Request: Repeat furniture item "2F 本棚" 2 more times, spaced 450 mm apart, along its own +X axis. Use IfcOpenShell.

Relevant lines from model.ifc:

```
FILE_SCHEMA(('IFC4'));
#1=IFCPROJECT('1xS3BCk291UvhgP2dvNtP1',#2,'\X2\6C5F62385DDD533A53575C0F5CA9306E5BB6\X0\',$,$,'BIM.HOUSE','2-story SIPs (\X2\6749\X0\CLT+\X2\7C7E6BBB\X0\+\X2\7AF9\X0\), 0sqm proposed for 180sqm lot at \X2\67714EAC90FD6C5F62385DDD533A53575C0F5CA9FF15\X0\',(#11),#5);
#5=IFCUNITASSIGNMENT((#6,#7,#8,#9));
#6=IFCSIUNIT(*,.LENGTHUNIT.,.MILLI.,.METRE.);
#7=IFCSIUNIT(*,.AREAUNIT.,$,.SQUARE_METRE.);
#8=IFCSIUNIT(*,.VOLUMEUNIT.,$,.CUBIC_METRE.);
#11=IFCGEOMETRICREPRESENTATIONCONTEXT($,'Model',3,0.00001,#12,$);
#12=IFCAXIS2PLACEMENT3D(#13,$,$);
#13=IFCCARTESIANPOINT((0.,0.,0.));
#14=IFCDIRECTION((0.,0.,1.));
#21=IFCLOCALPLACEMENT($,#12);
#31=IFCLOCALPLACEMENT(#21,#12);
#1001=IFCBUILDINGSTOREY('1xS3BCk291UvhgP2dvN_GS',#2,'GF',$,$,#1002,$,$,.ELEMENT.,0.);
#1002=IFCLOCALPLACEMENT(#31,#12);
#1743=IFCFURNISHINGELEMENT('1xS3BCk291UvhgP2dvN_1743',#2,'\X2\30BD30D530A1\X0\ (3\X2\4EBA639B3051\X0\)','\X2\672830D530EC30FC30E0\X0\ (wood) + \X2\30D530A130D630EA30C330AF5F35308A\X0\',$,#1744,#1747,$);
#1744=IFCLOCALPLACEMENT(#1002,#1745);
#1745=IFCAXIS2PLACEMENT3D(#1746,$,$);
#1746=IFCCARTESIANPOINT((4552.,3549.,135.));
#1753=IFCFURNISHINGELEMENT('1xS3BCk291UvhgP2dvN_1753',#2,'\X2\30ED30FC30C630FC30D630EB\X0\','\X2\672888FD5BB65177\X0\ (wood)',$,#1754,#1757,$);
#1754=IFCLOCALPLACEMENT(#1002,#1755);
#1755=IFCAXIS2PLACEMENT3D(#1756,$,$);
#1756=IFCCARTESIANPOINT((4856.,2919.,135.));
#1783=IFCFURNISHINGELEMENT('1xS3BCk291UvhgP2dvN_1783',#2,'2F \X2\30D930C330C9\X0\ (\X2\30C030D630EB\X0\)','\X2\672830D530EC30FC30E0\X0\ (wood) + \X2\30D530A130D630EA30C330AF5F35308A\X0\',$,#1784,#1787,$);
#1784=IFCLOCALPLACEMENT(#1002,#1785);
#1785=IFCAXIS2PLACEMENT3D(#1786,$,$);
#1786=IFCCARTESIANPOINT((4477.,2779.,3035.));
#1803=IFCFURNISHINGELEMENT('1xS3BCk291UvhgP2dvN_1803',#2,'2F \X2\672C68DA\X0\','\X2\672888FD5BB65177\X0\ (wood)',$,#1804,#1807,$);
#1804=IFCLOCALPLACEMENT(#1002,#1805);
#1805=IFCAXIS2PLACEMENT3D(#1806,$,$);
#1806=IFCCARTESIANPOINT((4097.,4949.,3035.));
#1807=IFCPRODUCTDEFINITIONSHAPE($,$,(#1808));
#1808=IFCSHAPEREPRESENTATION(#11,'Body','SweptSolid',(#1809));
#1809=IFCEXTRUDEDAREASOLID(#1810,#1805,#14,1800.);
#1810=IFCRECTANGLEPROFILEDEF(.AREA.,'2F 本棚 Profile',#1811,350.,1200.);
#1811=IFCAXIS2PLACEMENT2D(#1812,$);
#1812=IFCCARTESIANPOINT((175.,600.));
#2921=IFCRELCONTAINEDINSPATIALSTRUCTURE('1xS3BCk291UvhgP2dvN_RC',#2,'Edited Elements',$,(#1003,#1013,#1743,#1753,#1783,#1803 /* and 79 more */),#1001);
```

```python
import ifcopenshell
import ifcopenshell.api.geometry
import ifcopenshell.api.root
import ifcopenshell.util.element
import ifcopenshell.util.placement

model = ifcopenshell.open("model.ifc")


def reuse_history(source, copy):
    """copy_class also copies each property set's owner history, people and application; keep the originals."""
    for rel in copy.IsDefinedBy:
        if rel.is_a("IfcRelDefinesByProperties") and (history := rel.RelatingPropertyDefinition.OwnerHistory):
            rel.RelatingPropertyDefinition.OwnerHistory = source.OwnerHistory
            ifcopenshell.util.element.remove_deep2(model, history)


source = model.by_guid("1xS3BCk291UvhgP2dvN_1803")
base = ifcopenshell.util.placement.get_local_placement(source.ObjectPlacement)
step = base[:3, 0] * 450.0

for i in range(1, 3):
    copy = ifcopenshell.api.root.copy_class(model, product=source)
    copy.Representation = ifcopenshell.util.element.copy_deep(
        model, source.Representation, exclude=["IfcGeometricRepresentationContext", "IfcRepresentationMap"]
    )
    reuse_history(source, copy)
    matrix = base.copy()
    matrix[:3, 3] += i * step
    print("added at", matrix[:3, 3].round(3) + 0.0)
    ifcopenshell.api.geometry.edit_object_placement(model, product=copy, matrix=matrix, is_si=False)

model.write("model_v2.ifc")
```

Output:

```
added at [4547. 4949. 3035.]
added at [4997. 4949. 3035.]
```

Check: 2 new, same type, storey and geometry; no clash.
